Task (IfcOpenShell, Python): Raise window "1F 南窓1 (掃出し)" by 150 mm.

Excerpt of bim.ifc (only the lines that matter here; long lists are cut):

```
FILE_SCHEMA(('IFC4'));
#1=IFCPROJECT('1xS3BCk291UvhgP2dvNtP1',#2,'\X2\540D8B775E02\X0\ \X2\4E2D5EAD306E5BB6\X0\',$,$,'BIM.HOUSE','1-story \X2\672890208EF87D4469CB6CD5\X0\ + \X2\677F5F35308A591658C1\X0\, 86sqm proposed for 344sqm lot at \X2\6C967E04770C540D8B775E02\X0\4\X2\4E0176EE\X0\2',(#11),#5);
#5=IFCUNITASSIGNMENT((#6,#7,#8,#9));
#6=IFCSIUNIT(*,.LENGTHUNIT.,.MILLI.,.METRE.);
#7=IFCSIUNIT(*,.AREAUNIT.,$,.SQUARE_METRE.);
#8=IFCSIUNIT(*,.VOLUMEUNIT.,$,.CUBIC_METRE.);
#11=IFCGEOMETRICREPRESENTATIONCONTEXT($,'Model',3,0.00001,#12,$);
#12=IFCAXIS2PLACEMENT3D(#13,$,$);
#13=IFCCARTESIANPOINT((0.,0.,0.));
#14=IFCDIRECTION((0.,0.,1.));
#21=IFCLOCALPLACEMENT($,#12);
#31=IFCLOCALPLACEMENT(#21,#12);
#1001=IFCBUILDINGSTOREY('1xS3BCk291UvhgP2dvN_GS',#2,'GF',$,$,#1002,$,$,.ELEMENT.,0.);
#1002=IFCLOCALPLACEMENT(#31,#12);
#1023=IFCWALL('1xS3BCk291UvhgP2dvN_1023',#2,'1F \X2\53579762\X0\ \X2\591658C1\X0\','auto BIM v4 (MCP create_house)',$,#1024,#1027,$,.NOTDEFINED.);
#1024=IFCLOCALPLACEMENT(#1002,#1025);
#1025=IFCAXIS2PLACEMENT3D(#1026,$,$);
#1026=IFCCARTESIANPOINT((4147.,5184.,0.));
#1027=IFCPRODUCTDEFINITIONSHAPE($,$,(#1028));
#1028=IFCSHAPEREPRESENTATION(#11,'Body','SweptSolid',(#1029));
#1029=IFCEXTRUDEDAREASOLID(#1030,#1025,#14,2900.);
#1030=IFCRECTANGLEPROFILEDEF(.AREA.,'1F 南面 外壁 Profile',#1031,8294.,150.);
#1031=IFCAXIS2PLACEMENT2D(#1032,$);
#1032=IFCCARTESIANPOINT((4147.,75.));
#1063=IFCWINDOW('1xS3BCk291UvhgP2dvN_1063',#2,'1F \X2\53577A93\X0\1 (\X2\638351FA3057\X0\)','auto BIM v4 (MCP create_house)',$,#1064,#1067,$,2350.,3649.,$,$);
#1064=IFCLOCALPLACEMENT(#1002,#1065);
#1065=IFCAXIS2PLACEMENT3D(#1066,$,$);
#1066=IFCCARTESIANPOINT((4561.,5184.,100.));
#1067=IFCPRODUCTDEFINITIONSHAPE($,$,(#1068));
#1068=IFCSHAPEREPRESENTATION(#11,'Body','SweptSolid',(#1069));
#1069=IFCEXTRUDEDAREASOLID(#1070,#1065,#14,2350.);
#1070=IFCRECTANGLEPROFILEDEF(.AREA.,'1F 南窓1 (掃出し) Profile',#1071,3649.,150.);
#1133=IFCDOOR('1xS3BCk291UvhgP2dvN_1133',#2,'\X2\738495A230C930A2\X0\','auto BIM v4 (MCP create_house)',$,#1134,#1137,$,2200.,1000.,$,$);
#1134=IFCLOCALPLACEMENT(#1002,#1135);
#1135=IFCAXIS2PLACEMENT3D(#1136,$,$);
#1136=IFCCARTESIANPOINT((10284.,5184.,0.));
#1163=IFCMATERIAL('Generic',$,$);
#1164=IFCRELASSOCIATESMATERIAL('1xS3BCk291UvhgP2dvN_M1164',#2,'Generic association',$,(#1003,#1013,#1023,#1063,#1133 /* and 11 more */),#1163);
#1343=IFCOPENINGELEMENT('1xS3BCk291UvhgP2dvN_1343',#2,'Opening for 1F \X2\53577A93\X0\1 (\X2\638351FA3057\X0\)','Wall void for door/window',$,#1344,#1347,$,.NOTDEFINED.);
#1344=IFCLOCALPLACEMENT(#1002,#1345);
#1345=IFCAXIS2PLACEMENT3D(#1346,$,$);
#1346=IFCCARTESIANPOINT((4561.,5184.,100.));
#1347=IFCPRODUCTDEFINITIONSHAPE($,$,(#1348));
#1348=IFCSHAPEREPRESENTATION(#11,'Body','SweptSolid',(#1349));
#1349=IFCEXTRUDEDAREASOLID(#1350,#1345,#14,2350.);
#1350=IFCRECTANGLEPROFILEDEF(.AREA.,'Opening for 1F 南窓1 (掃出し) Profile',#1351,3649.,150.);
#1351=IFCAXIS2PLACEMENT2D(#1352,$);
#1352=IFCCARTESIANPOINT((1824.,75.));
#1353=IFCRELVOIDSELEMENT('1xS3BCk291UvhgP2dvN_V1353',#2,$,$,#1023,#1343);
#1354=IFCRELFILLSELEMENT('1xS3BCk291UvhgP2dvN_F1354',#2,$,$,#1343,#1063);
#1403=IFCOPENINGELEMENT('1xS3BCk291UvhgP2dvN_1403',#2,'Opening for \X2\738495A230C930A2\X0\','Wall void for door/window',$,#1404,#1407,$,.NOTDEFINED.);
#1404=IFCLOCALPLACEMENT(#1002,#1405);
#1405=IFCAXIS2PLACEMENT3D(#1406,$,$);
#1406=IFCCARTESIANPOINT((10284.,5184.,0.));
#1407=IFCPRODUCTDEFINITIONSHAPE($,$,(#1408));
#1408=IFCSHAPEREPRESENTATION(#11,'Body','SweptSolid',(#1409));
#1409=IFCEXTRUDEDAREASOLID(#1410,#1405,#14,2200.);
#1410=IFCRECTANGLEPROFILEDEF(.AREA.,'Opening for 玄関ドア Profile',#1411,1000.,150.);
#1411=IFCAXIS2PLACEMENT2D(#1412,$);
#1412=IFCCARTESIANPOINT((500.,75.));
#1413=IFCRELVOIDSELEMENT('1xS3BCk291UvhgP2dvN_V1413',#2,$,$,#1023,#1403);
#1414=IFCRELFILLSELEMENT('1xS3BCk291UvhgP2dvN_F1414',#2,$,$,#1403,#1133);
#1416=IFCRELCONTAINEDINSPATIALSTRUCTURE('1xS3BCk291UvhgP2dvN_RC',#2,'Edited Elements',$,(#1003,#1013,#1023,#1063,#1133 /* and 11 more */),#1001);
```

```python
import numpy as np
import ifcopenshell
import ifcopenshell.api.geometry
import ifcopenshell.util.placement
import ifcopenshell.util.unit

model = ifcopenshell.open("bim.ifc")
unit_scale = ifcopenshell.util.unit.calculate_unit_scale(model)

window = model.by_guid("1xS3BCk291UvhgP2dvN_1063")
opening = window.FillsVoids[0].RelatingOpeningElement
dz = 0.15 / unit_scale

shift = np.array([0.0, 0.0, dz])
# The window is not placed relative to its opening, so move both.
for product in (opening, window):
    matrix = ifcopenshell.util.placement.get_local_placement(product.ObjectPlacement)
    matrix[:3, 3] += shift
    ifcopenshell.api.geometry.edit_object_placement(model, product=product, matrix=matrix, is_si=False)

print(f"moved by {dz * unit_scale:+.3f} m")

model.write("bim-out.ifc")
```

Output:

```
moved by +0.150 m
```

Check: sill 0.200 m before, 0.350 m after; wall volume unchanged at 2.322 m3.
